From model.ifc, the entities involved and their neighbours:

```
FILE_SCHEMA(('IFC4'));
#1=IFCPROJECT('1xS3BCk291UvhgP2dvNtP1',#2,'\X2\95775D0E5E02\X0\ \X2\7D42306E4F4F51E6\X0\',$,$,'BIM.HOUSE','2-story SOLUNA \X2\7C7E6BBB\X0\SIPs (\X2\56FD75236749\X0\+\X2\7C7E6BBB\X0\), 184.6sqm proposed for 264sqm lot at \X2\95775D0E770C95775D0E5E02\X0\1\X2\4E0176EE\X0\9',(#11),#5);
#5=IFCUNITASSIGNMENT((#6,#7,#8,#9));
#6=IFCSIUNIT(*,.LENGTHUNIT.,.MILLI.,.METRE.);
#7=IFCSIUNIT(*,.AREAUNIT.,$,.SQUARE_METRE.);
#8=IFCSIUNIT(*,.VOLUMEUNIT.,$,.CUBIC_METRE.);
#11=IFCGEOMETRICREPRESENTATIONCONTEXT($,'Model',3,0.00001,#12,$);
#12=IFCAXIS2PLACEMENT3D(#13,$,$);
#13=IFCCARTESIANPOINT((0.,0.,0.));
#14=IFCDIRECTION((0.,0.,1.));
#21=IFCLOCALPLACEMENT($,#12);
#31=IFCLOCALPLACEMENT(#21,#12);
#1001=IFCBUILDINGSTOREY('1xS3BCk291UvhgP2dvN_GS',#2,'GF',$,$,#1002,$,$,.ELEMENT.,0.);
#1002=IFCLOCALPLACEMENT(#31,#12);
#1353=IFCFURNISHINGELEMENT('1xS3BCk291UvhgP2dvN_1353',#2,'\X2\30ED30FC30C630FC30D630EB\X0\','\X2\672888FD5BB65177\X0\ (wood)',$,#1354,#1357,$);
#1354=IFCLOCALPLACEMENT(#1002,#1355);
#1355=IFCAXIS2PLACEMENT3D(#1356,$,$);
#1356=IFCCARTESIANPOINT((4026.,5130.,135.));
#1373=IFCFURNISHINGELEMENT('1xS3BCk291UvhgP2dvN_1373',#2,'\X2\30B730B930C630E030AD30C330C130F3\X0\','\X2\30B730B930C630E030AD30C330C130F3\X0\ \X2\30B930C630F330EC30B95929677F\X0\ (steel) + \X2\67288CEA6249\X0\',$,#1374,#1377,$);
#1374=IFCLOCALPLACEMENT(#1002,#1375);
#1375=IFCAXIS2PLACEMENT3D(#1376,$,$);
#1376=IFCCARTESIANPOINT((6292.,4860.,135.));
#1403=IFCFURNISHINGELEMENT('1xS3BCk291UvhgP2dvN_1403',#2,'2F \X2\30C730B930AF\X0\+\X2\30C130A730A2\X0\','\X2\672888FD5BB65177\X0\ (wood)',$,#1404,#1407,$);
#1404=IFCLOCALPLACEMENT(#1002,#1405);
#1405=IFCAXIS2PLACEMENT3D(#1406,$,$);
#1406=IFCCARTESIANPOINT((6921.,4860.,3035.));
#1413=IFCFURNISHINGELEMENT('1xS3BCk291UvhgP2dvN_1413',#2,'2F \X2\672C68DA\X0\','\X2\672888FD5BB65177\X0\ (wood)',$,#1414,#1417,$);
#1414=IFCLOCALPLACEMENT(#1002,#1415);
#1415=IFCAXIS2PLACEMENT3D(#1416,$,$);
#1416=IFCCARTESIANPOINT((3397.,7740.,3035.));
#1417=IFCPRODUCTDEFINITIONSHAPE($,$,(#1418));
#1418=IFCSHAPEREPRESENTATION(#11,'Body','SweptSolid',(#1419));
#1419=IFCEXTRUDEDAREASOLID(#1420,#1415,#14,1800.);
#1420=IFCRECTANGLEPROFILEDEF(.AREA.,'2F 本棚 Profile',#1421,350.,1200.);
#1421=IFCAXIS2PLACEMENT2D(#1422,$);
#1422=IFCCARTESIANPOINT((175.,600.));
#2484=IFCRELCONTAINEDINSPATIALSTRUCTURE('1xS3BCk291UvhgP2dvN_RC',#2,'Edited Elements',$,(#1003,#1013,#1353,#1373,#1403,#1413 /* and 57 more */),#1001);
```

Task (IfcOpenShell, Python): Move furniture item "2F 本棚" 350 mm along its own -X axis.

```python
import ifcopenshell
import ifcopenshell.api.geometry
import ifcopenshell.util.placement
import ifcopenshell.util.unit

model = ifcopenshell.open("model.ifc")
unit_scale = ifcopenshell.util.unit.calculate_unit_scale(model)

item = model.by_guid("1xS3BCk291UvhgP2dvN_1413")
matrix = ifcopenshell.util.placement.get_local_placement(item.ObjectPlacement)
matrix[:3, 3] -= matrix[:3, 0] * 0.35 / unit_scale
ifcopenshell.api.geometry.edit_object_placement(model, product=item, matrix=matrix, is_si=False)

print(ifcopenshell.util.placement.get_local_placement(item.ObjectPlacement).round(3) + 0.0)

model.write("model_rev.ifc")
```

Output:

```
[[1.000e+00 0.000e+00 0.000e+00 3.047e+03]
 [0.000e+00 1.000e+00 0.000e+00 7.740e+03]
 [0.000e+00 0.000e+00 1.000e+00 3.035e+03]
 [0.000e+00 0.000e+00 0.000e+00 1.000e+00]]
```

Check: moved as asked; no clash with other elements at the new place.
